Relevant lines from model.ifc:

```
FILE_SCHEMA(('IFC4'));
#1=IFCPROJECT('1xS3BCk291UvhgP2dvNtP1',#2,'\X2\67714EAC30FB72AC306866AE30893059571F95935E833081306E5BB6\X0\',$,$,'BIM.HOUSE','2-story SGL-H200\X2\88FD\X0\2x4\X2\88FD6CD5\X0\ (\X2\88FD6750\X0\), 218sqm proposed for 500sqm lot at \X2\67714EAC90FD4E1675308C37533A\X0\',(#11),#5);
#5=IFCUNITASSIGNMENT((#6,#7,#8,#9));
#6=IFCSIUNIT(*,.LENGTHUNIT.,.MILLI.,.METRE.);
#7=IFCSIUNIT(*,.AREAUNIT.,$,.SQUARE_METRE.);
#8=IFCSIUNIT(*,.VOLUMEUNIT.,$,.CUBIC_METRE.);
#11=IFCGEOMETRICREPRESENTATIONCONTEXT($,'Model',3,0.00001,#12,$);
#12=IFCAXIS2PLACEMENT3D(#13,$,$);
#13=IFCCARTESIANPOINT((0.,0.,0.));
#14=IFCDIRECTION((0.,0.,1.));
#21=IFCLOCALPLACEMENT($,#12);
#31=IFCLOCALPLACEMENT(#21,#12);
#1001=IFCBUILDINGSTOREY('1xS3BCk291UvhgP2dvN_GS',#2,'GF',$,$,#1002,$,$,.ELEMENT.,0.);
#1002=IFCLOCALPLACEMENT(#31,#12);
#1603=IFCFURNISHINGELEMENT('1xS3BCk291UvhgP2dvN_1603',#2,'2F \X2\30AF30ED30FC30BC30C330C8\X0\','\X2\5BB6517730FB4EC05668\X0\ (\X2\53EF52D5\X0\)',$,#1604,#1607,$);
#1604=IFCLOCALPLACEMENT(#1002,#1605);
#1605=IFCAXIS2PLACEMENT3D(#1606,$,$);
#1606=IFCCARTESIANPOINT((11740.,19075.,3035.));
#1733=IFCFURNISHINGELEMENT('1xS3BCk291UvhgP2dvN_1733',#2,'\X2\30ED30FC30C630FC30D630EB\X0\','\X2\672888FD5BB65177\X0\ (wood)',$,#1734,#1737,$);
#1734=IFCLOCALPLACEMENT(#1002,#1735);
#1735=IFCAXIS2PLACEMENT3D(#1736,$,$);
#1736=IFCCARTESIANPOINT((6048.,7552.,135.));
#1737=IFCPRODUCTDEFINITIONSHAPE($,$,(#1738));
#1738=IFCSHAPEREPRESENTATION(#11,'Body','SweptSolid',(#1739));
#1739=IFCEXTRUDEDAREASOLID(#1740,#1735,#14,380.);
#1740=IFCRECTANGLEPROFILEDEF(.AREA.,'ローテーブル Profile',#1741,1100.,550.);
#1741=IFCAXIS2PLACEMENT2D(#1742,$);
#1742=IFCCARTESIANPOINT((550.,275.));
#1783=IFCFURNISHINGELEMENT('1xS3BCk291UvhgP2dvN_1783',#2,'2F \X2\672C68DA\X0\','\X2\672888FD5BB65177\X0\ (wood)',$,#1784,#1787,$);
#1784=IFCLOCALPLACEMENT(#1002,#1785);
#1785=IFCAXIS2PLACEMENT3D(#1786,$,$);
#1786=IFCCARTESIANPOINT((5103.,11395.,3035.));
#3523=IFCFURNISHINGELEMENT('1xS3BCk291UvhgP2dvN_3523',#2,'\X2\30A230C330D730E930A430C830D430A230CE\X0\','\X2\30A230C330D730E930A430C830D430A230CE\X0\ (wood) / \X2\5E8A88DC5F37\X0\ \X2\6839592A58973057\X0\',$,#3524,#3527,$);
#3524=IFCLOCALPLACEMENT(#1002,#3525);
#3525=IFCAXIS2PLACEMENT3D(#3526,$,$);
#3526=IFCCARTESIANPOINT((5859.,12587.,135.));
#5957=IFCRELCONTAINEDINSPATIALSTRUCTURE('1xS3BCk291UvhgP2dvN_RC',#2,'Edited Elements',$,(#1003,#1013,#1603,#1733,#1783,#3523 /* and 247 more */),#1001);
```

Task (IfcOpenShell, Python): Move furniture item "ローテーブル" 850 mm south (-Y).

```python
import ifcopenshell
import ifcopenshell.api.geometry
import ifcopenshell.util.placement
import ifcopenshell.util.unit

model = ifcopenshell.open("model.ifc")
unit_scale = ifcopenshell.util.unit.calculate_unit_scale(model)

item = model.by_guid("1xS3BCk291UvhgP2dvN_1733")
matrix = ifcopenshell.util.placement.get_local_placement(item.ObjectPlacement)
matrix[1, 3] -= 0.85 / unit_scale
ifcopenshell.api.geometry.edit_object_placement(model, product=item, matrix=matrix, is_si=False)

print(ifcopenshell.util.placement.get_local_placement(item.ObjectPlacement).round(3) + 0.0)

model.write("model-out.ifc")
```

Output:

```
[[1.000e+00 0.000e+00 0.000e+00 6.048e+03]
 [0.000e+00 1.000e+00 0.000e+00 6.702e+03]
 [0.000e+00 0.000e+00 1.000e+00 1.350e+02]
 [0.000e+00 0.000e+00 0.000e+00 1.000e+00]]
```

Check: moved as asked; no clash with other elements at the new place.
